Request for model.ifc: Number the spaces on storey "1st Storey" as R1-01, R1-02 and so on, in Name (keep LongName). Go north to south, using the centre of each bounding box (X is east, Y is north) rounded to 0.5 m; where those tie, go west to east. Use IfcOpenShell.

First a look at what the model holds.

```python
import ifcopenshell
import ifcopenshell.util.element
import ifcopenshell.util.placement

model = ifcopenshell.open("model.ifc")
print(model.schema)
storey = next(s for s in model.by_type("IfcBuildingStorey") if s.Name == "1st Storey")
spaces = [e for e in ifcopenshell.util.element.get_decomposition(storey) if e.is_a("IfcSpace")]
for e in sorted(spaces, key=lambda e: e.id()):
    origin = ifcopenshell.util.placement.get_local_placement(e.ObjectPlacement)[:3, 3]
    print(e.id(), e.Name, e.LongName, origin.round(2) + 0.0, sep=" | ")
```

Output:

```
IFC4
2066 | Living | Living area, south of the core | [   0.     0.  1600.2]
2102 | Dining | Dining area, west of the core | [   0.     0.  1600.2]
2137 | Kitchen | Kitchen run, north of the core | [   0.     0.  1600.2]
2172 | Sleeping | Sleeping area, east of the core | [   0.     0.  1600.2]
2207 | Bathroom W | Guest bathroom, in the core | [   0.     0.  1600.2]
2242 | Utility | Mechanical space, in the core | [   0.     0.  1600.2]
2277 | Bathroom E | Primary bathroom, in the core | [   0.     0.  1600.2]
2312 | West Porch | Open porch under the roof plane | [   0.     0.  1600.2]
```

```python
import ifcopenshell
import ifcopenshell.geom
import ifcopenshell.util.element
import ifcopenshell.util.shape

model = ifcopenshell.open("model.ifc")
settings = ifcopenshell.geom.settings()
settings.set("use-world-coords", True)


def centre(element):
    shape = ifcopenshell.geom.create_shape(settings, element)
    return ifcopenshell.util.shape.get_bbox_centroid(shape.geometry)


storey = next(s for s in model.by_type("IfcBuildingStorey") if s.Name == "1st Storey")
spaces = [e for e in ifcopenshell.util.element.get_decomposition(storey) if e.is_a("IfcSpace")]

# Insertion points can sit at a corner or the storey origin, so sort by the geometry (in metres).
centres = {e: centre(e) for e in spaces}
spaces.sort(key=lambda e: (-round(centres[e][1] / 0.5), centres[e][0]))

for i, e in enumerate(spaces, start=1):
    number = f"R1-{i:02d}"
    e.Name = number
    print(e.id(), number)

model.write("model_updated.ifc")
```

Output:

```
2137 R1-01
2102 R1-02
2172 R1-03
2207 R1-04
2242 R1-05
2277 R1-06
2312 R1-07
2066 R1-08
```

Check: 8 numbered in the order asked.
